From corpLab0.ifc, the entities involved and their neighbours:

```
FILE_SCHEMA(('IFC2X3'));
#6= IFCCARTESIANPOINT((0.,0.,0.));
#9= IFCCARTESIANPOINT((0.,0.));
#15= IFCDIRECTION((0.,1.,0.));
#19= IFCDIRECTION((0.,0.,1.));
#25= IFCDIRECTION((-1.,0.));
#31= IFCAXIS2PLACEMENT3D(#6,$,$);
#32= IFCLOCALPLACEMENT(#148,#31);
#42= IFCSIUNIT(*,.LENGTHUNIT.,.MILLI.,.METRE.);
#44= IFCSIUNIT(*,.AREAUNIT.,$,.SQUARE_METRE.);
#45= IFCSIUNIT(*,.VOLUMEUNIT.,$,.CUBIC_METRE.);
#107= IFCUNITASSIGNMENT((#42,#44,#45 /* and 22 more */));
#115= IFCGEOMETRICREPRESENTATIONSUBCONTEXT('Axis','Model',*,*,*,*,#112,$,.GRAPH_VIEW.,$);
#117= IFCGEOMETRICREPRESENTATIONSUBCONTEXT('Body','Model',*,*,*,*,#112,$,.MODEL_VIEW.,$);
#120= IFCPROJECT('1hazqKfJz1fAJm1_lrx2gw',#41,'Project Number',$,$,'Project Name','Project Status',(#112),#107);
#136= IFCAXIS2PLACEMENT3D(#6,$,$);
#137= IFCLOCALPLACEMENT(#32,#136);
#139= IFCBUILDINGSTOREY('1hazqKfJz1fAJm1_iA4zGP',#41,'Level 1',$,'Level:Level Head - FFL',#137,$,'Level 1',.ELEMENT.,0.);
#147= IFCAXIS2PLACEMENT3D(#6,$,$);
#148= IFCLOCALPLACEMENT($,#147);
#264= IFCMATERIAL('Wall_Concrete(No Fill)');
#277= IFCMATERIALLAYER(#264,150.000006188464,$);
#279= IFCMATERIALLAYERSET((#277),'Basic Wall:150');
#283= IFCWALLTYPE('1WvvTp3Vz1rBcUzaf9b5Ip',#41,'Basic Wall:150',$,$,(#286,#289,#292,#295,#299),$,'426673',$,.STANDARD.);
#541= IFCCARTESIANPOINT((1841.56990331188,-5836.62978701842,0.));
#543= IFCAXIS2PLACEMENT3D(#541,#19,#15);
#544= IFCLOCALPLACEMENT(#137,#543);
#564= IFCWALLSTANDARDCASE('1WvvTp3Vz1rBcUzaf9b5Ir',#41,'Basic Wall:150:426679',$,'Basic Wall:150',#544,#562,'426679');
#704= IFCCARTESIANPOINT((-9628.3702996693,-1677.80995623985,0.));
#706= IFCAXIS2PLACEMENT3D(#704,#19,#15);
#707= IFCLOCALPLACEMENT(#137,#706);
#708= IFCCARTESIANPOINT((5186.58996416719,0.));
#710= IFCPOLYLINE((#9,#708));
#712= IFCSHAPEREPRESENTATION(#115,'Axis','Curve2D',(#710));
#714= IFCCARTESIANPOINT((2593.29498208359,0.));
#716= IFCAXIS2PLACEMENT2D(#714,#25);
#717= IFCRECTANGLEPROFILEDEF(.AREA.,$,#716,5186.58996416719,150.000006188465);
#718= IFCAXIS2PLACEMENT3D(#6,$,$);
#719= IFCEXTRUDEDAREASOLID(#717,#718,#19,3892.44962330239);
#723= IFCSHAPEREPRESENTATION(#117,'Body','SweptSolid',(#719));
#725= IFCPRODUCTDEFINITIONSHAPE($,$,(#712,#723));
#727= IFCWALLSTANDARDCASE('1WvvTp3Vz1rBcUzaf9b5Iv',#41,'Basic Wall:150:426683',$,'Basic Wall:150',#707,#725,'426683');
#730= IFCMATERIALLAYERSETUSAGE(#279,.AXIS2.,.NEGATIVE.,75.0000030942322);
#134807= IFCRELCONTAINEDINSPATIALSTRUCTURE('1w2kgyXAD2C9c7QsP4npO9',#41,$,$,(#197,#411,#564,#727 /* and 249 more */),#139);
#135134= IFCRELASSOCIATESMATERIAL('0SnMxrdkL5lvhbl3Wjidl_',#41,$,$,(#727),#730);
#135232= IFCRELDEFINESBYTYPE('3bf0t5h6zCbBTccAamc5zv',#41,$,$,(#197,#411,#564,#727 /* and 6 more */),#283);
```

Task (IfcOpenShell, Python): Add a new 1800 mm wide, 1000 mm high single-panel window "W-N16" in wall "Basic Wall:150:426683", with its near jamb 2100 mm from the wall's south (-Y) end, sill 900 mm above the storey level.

```python
import numpy as np
import ifcopenshell
import ifcopenshell.api.feature
import ifcopenshell.api.geometry
import ifcopenshell.api.root
import ifcopenshell.api.spatial
import ifcopenshell.api.type
import ifcopenshell.geom
import ifcopenshell.util.element
import ifcopenshell.util.placement
import ifcopenshell.util.representation
import ifcopenshell.util.shape
import ifcopenshell.util.unit

model = ifcopenshell.open("corpLab0.ifc")
unit_scale = ifcopenshell.util.unit.calculate_unit_scale(model)
settings = ifcopenshell.geom.settings()


def volume(element):
    """Net volume in cubic metres, openings subtracted."""
    shape = ifcopenshell.geom.create_shape(settings, element)
    return ifcopenshell.util.shape.get_volume(shape.geometry)


wall = model.by_guid("1WvvTp3Vz1rBcUzaf9b5Iv")
storey = ifcopenshell.util.element.get_container(wall, ifc_class="IfcBuildingStorey")
context = ifcopenshell.util.representation.get_context(model, "Model", "Body", "MODEL_VIEW")
before = volume(wall)

width, height, from_end, sill = 1.8, 1, 2.1, 0.9  # metres

# The wall runs along its own X axis, and the end named is its -X end.
wall_shape = ifcopenshell.geom.create_shape(settings, wall)
x, y, z = ifcopenshell.util.shape.get_vertices(wall_shape.geometry).T
start = x.min() + from_end
face, thickness = float(y.min()), float(y.max() - y.min())
wall_matrix = ifcopenshell.util.placement.get_local_placement(wall.ObjectPlacement)
level = ifcopenshell.util.placement.get_local_placement(storey.ObjectPlacement)[2, 3]


def in_wall(x, y):
    """Placement at x, y metres in the wall's axes, at sill height."""
    matrix = wall_matrix.copy()
    matrix[:, 3] = wall_matrix @ np.array([x / unit_scale, y / unit_scale, 0.0, 1.0])
    matrix[2, 3] = level + sill / unit_scale
    return matrix


# Opening: a box that overshoots both wall faces by 50 mm.
opening = ifcopenshell.api.root.create_entity(model, ifc_class="IfcOpeningElement")
box = ifcopenshell.api.geometry.add_wall_representation(
    model, context=context, length=width, height=height, thickness=thickness + 0.1
)
ifcopenshell.api.geometry.assign_representation(model, product=opening, representation=box)
ifcopenshell.api.geometry.edit_object_placement(model, product=opening, matrix=in_wall(start, face - 0.05), is_si=False)
ifcopenshell.api.feature.add_feature(model, feature=opening, element=wall)

window = ifcopenshell.api.root.create_entity(model, ifc_class="IfcWindow", name="W-N16")
window.OverallWidth, window.OverallHeight = width / unit_scale, height / unit_scale
body = ifcopenshell.api.geometry.add_window_representation(
    model,
    context=context,
    overall_width=window.OverallWidth,
    overall_height=window.OverallHeight,
    partition_type="SINGLE_PANEL",
)
ifcopenshell.api.geometry.assign_representation(model, product=window, representation=body)
ifcopenshell.api.spatial.assign_container(model, products=[window], relating_structure=storey)
fills = ifcopenshell.api.feature.add_filling(model, opening=opening, element=window)
fills.OwnerHistory = window.OwnerHistory  # required in IFC2X3

# IFC2X3 keeps the operation on the window style.
style = ifcopenshell.api.root.create_entity(model, ifc_class="IfcWindowStyle", name="W-N16")
style.OperationType, style.ConstructionType = "SINGLE_PANEL", "NOTDEFINED"
style.ParameterTakesPrecedence = style.Sizeable = False
ifcopenshell.api.type.assign_type(model, related_objects=[window], relating_type=style)

# Centre the window in the wall's thickness.
ifcopenshell.api.geometry.edit_object_placement(model, product=window, matrix=in_wall(start, face), is_si=False)
window_shape = ifcopenshell.geom.create_shape(settings, window)
depth = ifcopenshell.util.shape.get_vertices(window_shape.geometry)[:, 1]
offset = face + thickness / 2 - (depth.min() + depth.max()) / 2
ifcopenshell.api.geometry.edit_object_placement(model, product=window, matrix=in_wall(start, offset), is_si=False)

after = volume(wall)

print(f"wall volume {before:.3f} -> {after:.3f} m3")

model.write("corpLab0_v2.ifc")
```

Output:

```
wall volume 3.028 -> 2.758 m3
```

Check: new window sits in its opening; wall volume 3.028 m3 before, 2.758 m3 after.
